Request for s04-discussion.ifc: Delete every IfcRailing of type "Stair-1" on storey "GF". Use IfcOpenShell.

First a look at what the model holds.

```python
import ifcopenshell
import ifcopenshell.util.element

model = ifcopenshell.open("s04-discussion.ifc")
print(model.schema)
storey = next(s for s in model.by_type("IfcBuildingStorey") if s.Name == "GF")
railings = [e for e in ifcopenshell.util.element.get_decomposition(storey) if e.is_a("IfcRailing")]
seen = {}
for e in railings:
    element_type = ifcopenshell.util.element.get_type(e)
    name = element_type.Name if element_type not in (None, e) else None
    seen[name] = seen.get(name, 0) + 1
for name, count in sorted(seen.items(), key=str):
    print(count, "x", name)
```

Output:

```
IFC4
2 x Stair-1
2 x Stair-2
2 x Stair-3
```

```python
import ifcopenshell
import ifcopenshell.api.root
import ifcopenshell.util.element

model = ifcopenshell.open("s04-discussion.ifc")

storey = next(s for s in model.by_type("IfcBuildingStorey") if s.Name == "GF")
railings = [e for e in ifcopenshell.util.element.get_decomposition(storey) if e.is_a("IfcRailing")]
targets = [e for e in railings if (t := ifcopenshell.util.element.get_type(e)) not in (None, e) and t.Name == "Stair-1"]

for e in targets:
    ifcopenshell.api.root.remove_product(model, product=e)
print(len(targets), "removed")

model.write("s04-discussion_updated.ifc")
```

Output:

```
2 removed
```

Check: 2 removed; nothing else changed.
